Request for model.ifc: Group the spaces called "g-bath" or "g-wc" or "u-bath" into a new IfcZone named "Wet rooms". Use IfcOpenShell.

First a look at what the model holds.

```python
import ifcopenshell

model = ifcopenshell.open("model.ifc")
print(model.schema)
seen = {}
for space in model.by_type("IfcSpace"):
    seen[space.LongName] = seen.get(space.LongName, 0) + 1
for name, count in sorted(seen.items(), key=str):
    print(count, "x", name)
print("zones:", [z.Name for z in model.by_type("IfcZone")][:20])
```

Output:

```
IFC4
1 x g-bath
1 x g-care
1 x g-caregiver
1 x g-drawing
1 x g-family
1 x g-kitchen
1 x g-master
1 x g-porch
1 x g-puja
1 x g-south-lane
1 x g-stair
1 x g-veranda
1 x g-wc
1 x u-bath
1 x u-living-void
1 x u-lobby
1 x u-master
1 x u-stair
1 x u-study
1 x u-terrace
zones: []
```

```python
import ifcopenshell
import ifcopenshell.api.group
import ifcopenshell.api.root

model = ifcopenshell.open("model.ifc")

names = {"g-bath", "g-wc", "u-bath"}
spaces = [s for s in model.by_type("IfcSpace") if s.LongName in names]

zone = ifcopenshell.api.root.create_entity(model, ifc_class="IfcZone", name="Wet rooms")
ifcopenshell.api.group.assign_group(model, products=spaces, group=zone)
print(len(spaces), "spaces in", zone.Name)

model.write("model_v2.ifc")
```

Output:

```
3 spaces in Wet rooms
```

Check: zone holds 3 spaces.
